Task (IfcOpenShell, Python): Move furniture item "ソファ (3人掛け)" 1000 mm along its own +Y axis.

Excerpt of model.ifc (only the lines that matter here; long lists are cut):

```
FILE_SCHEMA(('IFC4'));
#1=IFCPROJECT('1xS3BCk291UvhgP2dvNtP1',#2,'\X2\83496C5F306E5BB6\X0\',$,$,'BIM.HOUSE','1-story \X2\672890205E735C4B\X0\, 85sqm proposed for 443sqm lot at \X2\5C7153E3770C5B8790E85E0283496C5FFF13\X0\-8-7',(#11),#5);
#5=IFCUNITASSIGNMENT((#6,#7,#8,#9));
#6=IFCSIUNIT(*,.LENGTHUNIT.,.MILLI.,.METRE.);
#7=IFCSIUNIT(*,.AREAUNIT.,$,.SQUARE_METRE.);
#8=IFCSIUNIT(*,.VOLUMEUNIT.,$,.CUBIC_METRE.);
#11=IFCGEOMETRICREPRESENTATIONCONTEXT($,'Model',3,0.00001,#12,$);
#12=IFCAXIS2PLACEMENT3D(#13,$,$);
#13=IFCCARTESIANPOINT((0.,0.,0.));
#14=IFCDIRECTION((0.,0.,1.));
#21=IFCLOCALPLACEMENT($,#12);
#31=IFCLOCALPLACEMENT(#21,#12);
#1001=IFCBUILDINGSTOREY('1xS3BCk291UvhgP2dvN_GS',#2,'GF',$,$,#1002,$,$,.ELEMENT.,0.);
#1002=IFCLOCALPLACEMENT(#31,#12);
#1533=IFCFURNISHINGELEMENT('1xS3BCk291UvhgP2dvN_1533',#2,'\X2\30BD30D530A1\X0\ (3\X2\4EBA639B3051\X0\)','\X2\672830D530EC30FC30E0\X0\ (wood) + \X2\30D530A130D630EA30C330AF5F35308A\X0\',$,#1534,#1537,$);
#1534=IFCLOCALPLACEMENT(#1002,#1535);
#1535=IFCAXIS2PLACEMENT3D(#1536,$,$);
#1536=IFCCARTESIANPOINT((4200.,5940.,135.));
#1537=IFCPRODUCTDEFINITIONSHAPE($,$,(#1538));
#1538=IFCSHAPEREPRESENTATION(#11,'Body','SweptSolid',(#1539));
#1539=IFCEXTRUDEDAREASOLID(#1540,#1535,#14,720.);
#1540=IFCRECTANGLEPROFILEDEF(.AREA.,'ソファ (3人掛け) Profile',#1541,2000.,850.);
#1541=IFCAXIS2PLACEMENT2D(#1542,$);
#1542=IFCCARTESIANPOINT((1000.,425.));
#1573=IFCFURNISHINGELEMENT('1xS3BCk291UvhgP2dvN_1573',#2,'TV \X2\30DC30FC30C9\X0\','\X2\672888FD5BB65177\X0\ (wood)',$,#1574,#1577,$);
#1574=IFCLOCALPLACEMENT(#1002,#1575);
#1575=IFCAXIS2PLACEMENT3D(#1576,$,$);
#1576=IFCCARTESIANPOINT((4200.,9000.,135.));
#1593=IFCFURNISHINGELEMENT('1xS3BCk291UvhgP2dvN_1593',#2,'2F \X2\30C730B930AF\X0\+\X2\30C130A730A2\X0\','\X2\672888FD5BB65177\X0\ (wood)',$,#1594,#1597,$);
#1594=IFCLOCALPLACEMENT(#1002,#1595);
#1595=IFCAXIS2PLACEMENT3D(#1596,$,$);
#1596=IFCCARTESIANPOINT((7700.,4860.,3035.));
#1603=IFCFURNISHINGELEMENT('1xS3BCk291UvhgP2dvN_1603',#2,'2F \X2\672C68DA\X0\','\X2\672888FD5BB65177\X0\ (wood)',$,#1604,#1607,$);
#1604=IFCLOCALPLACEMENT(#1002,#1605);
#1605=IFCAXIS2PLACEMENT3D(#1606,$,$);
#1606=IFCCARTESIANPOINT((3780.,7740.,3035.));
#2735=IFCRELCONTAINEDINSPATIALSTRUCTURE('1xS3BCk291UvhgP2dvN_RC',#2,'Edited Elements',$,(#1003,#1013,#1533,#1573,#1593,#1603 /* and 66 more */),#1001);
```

```python
import ifcopenshell
import ifcopenshell.api.geometry
import ifcopenshell.util.placement

model = ifcopenshell.open("model.ifc")

item = model.by_guid("1xS3BCk291UvhgP2dvN_1533")
matrix = ifcopenshell.util.placement.get_local_placement(item.ObjectPlacement)
matrix[:3, 3] += matrix[:3, 1] * 1000.0
ifcopenshell.api.geometry.edit_object_placement(model, product=item, matrix=matrix, is_si=False)

print(ifcopenshell.util.placement.get_local_placement(item.ObjectPlacement).round(3) + 0.0)

model.write("model_edited.ifc")
```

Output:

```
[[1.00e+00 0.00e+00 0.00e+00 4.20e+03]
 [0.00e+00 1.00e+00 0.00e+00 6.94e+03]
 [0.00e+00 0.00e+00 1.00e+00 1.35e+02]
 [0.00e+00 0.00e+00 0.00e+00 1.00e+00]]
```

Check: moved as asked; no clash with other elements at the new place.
